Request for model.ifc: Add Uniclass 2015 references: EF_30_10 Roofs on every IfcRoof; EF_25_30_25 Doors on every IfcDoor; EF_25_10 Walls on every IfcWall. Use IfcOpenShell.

First a look at what the model holds.

```python
import ifcopenshell

model = ifcopenshell.open("model.ifc")
print(model.schema)
print("classifications:", [c.Name for c in model.by_type("IfcClassification")])
for ifc_class in ("IfcDoor", "IfcRoof", "IfcStair", "IfcWall", "IfcWindow"):
    print(ifc_class, len(model.by_type(ifc_class)))
```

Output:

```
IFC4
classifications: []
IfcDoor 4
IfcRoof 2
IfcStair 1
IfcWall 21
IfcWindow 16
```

```python
import ifcopenshell
import ifcopenshell.api.classification

model = ifcopenshell.open("model.ifc")

system = ifcopenshell.api.classification.add_classification(model, classification="Uniclass 2015")

codes = {
    "IfcRoof": ("EF_30_10", "Roofs"),
    "IfcDoor": ("EF_25_30_25", "Doors"),
    "IfcWall": ("EF_25_10", "Walls"),
}
for ifc_class, (code, name) in codes.items():
    products = model.by_type(ifc_class)
    ifcopenshell.api.classification.add_reference(
        model, products=products, classification=system, identification=code, name=name
    )
    print(code, len(products))

model.write("model_v2.ifc")
```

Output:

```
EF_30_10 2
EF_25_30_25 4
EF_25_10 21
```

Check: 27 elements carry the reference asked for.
